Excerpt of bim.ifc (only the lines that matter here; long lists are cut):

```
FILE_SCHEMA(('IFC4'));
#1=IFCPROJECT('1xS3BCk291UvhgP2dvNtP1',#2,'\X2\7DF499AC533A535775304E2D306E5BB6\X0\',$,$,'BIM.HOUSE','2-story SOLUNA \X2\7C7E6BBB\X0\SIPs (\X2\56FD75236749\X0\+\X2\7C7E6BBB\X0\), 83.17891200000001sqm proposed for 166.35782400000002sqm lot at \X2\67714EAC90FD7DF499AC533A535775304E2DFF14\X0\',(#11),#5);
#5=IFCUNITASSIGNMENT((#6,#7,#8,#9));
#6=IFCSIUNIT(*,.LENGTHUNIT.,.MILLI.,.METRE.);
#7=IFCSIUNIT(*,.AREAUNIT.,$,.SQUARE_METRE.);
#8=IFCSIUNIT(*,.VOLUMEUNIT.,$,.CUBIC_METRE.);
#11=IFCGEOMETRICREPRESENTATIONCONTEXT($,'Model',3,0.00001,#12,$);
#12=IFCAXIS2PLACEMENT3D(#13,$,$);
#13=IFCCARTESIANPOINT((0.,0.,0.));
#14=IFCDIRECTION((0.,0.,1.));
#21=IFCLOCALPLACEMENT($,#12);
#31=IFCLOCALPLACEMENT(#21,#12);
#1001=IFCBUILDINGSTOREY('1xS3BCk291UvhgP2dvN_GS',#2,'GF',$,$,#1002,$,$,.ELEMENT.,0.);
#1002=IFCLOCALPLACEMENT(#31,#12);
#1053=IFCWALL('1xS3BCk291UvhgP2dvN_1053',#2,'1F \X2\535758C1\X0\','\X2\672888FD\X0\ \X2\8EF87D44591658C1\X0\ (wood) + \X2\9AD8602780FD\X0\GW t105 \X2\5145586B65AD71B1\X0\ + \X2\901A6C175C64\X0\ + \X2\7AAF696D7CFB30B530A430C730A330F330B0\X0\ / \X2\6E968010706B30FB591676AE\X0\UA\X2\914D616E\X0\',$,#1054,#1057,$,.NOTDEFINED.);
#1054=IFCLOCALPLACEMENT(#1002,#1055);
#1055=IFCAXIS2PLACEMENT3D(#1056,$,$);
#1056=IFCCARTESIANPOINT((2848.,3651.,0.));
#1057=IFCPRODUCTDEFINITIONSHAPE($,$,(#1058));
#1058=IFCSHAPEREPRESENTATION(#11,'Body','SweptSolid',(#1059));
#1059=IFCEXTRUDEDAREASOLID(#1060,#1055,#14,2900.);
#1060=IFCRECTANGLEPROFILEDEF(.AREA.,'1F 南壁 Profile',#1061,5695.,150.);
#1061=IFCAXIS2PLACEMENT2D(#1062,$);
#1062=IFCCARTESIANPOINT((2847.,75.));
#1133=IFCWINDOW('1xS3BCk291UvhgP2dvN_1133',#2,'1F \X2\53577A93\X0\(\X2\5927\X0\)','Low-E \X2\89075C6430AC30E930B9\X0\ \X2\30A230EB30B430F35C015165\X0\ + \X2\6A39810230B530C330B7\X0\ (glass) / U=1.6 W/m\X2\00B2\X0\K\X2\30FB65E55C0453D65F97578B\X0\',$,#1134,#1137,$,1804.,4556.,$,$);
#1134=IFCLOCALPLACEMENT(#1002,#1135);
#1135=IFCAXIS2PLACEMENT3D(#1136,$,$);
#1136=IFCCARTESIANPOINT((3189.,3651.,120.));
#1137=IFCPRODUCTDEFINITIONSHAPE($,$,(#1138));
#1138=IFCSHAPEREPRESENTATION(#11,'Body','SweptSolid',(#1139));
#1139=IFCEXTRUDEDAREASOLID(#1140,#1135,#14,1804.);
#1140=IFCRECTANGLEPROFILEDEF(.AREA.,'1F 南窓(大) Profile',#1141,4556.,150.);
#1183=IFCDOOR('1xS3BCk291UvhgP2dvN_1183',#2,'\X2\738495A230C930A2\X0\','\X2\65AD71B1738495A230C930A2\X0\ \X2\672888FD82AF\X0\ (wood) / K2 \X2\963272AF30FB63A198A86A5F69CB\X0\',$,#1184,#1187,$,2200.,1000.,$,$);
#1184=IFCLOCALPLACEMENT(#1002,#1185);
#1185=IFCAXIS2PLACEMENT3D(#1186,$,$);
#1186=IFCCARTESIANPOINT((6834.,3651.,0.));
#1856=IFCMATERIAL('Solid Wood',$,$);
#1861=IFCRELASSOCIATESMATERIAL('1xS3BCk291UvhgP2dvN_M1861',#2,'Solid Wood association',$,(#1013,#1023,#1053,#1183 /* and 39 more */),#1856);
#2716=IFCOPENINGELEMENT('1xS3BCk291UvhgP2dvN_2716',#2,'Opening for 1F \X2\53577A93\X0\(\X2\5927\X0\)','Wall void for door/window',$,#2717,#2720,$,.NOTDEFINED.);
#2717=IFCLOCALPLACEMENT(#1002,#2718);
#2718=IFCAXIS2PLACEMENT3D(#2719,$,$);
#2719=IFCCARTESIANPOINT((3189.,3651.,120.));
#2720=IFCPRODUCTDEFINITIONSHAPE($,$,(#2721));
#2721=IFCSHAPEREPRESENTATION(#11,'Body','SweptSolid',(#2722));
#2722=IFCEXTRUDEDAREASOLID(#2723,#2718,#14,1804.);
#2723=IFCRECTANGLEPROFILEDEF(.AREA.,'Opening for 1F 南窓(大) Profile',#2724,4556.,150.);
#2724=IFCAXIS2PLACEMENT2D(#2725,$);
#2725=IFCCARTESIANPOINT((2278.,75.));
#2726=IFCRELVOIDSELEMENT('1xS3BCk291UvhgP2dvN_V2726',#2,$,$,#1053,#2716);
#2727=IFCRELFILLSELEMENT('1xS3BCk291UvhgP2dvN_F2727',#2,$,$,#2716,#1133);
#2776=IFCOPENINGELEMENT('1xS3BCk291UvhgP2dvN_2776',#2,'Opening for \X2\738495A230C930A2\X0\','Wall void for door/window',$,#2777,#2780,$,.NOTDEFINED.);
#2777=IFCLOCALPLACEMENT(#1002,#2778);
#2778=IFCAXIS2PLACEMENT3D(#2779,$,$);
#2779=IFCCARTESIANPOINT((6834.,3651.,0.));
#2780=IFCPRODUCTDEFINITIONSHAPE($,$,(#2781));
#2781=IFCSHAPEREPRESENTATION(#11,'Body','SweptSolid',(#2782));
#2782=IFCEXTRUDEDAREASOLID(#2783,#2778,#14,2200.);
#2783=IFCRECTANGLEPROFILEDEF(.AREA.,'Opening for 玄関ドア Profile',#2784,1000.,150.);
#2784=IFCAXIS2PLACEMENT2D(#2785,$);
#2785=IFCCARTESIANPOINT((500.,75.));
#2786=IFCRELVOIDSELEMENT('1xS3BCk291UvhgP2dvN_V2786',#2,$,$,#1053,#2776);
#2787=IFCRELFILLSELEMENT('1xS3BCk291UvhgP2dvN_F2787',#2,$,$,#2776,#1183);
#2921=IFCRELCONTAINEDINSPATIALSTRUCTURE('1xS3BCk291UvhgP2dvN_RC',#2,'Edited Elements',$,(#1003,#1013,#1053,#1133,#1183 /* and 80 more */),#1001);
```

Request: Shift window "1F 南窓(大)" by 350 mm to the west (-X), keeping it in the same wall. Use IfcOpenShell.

```python
import ifcopenshell
import ifcopenshell.api.geometry
import ifcopenshell.util.placement
import ifcopenshell.util.unit

model = ifcopenshell.open("bim.ifc")
unit_scale = ifcopenshell.util.unit.calculate_unit_scale(model)

window = model.by_guid("1xS3BCk291UvhgP2dvN_1133")
opening = window.FillsVoids[0].RelatingOpeningElement
wall = opening.VoidsElements[0].RelatingBuildingElement

wall_matrix = ifcopenshell.util.placement.get_local_placement(wall.ObjectPlacement)
shift = wall_matrix[:3, 0] * -0.35 / unit_scale
before = ifcopenshell.util.placement.get_local_placement(window.ObjectPlacement)[:3, 3].copy()

# The window is not placed relative to its opening, so move both.
for product in (opening, window):
    matrix = ifcopenshell.util.placement.get_local_placement(product.ObjectPlacement)
    matrix[:3, 3] += shift
    ifcopenshell.api.geometry.edit_object_placement(model, product=product, matrix=matrix, is_si=False)

after = ifcopenshell.util.placement.get_local_placement(window.ObjectPlacement)[:3, 3]
print("window moved by", (after - before).round(3) + 0.0)

model.write("bim_updated.ifc")
```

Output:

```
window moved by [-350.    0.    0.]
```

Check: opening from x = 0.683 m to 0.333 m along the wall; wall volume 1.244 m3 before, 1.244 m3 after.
